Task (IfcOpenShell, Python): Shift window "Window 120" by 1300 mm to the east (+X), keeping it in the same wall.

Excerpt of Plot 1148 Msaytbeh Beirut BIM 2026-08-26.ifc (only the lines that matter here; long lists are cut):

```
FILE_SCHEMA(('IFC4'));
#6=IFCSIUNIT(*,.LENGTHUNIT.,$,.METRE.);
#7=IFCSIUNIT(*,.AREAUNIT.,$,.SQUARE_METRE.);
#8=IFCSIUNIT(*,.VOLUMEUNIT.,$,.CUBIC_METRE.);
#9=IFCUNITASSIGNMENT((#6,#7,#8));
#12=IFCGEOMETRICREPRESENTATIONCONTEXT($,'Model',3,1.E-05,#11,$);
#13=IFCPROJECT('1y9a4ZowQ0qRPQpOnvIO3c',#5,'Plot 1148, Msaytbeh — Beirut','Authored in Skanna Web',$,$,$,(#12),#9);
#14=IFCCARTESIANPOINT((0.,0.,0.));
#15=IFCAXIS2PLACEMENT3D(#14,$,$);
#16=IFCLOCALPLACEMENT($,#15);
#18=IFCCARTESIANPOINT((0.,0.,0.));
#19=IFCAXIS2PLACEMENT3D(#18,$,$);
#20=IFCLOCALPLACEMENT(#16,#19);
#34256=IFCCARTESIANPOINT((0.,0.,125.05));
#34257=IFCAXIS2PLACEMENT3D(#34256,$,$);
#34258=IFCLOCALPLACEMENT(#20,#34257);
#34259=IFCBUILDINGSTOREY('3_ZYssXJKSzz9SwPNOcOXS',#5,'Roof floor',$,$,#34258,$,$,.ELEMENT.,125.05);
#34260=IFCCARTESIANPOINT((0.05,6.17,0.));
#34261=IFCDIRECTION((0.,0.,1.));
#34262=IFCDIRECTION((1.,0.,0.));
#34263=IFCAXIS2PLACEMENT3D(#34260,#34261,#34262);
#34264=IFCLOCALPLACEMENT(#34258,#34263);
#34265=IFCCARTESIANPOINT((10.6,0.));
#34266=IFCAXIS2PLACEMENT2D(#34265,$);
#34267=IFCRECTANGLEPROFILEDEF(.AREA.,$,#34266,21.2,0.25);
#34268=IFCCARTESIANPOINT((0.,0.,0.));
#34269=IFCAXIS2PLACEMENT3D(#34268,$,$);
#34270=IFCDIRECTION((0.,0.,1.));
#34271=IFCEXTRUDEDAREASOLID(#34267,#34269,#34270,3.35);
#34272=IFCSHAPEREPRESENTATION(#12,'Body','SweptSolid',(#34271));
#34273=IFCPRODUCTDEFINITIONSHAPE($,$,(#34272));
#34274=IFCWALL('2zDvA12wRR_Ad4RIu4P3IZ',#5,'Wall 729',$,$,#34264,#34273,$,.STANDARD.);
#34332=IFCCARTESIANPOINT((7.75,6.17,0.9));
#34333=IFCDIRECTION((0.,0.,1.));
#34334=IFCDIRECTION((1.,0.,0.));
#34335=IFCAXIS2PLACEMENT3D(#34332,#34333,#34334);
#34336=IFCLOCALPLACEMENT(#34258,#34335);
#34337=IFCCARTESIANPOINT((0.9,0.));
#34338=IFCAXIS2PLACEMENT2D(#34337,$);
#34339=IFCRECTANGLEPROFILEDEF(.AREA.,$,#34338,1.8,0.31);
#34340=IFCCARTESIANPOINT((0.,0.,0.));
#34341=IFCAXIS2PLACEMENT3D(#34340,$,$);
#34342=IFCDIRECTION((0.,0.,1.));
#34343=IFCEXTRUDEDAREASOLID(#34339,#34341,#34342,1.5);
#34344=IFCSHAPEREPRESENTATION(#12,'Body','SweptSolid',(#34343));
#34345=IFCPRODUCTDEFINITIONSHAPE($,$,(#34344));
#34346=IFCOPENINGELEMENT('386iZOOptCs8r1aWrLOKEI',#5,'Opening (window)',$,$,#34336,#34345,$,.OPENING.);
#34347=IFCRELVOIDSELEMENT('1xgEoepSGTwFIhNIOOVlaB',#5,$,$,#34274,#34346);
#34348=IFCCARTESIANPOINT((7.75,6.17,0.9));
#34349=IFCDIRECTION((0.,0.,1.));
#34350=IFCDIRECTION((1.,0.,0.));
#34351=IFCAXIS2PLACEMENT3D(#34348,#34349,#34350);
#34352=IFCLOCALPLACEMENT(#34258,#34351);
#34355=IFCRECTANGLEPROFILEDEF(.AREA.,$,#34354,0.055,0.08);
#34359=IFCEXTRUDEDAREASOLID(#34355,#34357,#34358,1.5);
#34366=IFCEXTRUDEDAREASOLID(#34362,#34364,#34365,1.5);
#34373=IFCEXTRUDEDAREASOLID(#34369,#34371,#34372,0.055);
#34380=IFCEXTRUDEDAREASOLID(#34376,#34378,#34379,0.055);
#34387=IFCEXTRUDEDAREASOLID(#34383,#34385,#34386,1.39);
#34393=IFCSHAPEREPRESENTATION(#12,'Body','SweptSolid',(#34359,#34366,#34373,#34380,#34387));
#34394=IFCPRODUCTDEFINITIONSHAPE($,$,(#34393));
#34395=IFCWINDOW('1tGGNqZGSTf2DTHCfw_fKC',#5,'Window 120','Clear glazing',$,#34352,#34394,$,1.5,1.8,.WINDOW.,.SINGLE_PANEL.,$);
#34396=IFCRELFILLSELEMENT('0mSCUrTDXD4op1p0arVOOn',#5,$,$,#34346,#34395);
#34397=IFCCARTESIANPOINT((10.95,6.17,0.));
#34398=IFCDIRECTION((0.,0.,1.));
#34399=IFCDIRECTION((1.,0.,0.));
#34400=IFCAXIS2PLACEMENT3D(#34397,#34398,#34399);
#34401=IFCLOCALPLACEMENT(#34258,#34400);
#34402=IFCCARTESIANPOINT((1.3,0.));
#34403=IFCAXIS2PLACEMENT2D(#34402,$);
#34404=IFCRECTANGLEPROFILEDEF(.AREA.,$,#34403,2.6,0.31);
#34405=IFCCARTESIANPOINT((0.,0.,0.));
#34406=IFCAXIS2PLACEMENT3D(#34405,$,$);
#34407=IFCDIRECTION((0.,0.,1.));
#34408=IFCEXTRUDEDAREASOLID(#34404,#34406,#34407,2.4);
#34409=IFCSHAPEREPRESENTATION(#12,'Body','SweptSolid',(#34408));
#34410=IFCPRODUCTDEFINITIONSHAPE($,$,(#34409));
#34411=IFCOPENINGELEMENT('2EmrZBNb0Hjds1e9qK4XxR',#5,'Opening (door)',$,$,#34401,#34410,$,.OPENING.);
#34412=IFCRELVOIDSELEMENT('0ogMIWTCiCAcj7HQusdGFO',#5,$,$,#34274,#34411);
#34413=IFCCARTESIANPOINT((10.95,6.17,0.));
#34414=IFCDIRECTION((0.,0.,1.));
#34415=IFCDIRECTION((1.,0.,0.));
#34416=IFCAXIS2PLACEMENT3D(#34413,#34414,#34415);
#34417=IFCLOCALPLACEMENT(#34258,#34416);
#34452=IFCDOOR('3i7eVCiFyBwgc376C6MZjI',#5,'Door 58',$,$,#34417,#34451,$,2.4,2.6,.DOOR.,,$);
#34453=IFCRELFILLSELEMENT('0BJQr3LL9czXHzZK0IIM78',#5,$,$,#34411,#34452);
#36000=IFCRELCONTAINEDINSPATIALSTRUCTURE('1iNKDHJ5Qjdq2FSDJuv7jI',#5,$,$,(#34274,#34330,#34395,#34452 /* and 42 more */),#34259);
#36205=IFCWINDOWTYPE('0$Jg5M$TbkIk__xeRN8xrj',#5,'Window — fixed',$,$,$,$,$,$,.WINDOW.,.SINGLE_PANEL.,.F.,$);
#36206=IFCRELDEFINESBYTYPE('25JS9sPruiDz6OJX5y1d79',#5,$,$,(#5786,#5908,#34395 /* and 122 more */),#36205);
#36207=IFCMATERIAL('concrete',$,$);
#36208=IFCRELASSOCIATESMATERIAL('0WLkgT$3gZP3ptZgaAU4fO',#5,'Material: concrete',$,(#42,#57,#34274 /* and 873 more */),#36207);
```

```python
import ifcopenshell
import ifcopenshell.api.geometry
import ifcopenshell.util.placement
import ifcopenshell.util.unit

model = ifcopenshell.open("Plot 1148 Msaytbeh Beirut BIM 2026-08-26.ifc")
unit_scale = ifcopenshell.util.unit.calculate_unit_scale(model)

window = model.by_guid("1tGGNqZGSTf2DTHCfw_fKC")
opening = window.FillsVoids[0].RelatingOpeningElement
wall = opening.VoidsElements[0].RelatingBuildingElement

wall_matrix = ifcopenshell.util.placement.get_local_placement(wall.ObjectPlacement)
shift = wall_matrix[:3, 0] * 1.3 / unit_scale
before = ifcopenshell.util.placement.get_local_placement(window.ObjectPlacement)[:3, 3].copy()

# The window is not placed relative to its opening, so move both.
for product in (opening, window):
    matrix = ifcopenshell.util.placement.get_local_placement(product.ObjectPlacement)
    matrix[:3, 3] += shift
    ifcopenshell.api.geometry.edit_object_placement(model, product=product, matrix=matrix, is_si=False)

after = ifcopenshell.util.placement.get_local_placement(window.ObjectPlacement)[:3, 3]
print("window moved by", (after - before).round(3) + 0.0)

model.write("Plot 1148 Msaytbeh Beirut BIM 2026-08-26_edited.ifc")
```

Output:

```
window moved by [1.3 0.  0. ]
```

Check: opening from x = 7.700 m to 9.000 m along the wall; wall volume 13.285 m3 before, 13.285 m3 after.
